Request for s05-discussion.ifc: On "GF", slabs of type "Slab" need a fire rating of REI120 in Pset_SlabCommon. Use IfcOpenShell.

First a look at what the model holds.

```python
import ifcopenshell
import ifcopenshell.util.element

model = ifcopenshell.open("s05-discussion.ifc")
print(model.schema)
storey = next(s for s in model.by_type("IfcBuildingStorey") if s.Name == "GF")
slabs = [e for e in ifcopenshell.util.element.get_decomposition(storey) if e.is_a("IfcSlab")]
seen = {}
for e in slabs:
    element_type = ifcopenshell.util.element.get_type(e)
    key = (element_type.Name if element_type != e and element_type else None, ifcopenshell.util.element.get_pset(e, "Pset_SlabCommon", "FireRating"))
    seen[key] = seen.get(key, 0) + 1
for (name, value), count in sorted(seen.items(), key=str):
    print(count, "x", name, "|", value)
```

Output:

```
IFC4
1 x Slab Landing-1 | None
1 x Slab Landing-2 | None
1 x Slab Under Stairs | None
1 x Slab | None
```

```python
import ifcopenshell
import ifcopenshell.api.pset
import ifcopenshell.util.element

model = ifcopenshell.open("s05-discussion.ifc")

storey = next(s for s in model.by_type("IfcBuildingStorey") if s.Name == "GF")
slabs = [e for e in ifcopenshell.util.element.get_decomposition(storey) if e.is_a("IfcSlab")]

count = 0
for e in slabs:
    element_type = ifcopenshell.util.element.get_type(e)
    if element_type in (None, e) or element_type.Name != "Slab":
        continue
    # add_pset returns the element's existing set when there is one.
    pset = ifcopenshell.api.pset.add_pset(model, product=e, name="Pset_SlabCommon")
    ifcopenshell.api.pset.edit_pset(model, pset=pset, properties={"FireRating": "REI120"})
    count += 1

print(count, "slabs updated")

model.write("s05-discussion_edited.ifc")
```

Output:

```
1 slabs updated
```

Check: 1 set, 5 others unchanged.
